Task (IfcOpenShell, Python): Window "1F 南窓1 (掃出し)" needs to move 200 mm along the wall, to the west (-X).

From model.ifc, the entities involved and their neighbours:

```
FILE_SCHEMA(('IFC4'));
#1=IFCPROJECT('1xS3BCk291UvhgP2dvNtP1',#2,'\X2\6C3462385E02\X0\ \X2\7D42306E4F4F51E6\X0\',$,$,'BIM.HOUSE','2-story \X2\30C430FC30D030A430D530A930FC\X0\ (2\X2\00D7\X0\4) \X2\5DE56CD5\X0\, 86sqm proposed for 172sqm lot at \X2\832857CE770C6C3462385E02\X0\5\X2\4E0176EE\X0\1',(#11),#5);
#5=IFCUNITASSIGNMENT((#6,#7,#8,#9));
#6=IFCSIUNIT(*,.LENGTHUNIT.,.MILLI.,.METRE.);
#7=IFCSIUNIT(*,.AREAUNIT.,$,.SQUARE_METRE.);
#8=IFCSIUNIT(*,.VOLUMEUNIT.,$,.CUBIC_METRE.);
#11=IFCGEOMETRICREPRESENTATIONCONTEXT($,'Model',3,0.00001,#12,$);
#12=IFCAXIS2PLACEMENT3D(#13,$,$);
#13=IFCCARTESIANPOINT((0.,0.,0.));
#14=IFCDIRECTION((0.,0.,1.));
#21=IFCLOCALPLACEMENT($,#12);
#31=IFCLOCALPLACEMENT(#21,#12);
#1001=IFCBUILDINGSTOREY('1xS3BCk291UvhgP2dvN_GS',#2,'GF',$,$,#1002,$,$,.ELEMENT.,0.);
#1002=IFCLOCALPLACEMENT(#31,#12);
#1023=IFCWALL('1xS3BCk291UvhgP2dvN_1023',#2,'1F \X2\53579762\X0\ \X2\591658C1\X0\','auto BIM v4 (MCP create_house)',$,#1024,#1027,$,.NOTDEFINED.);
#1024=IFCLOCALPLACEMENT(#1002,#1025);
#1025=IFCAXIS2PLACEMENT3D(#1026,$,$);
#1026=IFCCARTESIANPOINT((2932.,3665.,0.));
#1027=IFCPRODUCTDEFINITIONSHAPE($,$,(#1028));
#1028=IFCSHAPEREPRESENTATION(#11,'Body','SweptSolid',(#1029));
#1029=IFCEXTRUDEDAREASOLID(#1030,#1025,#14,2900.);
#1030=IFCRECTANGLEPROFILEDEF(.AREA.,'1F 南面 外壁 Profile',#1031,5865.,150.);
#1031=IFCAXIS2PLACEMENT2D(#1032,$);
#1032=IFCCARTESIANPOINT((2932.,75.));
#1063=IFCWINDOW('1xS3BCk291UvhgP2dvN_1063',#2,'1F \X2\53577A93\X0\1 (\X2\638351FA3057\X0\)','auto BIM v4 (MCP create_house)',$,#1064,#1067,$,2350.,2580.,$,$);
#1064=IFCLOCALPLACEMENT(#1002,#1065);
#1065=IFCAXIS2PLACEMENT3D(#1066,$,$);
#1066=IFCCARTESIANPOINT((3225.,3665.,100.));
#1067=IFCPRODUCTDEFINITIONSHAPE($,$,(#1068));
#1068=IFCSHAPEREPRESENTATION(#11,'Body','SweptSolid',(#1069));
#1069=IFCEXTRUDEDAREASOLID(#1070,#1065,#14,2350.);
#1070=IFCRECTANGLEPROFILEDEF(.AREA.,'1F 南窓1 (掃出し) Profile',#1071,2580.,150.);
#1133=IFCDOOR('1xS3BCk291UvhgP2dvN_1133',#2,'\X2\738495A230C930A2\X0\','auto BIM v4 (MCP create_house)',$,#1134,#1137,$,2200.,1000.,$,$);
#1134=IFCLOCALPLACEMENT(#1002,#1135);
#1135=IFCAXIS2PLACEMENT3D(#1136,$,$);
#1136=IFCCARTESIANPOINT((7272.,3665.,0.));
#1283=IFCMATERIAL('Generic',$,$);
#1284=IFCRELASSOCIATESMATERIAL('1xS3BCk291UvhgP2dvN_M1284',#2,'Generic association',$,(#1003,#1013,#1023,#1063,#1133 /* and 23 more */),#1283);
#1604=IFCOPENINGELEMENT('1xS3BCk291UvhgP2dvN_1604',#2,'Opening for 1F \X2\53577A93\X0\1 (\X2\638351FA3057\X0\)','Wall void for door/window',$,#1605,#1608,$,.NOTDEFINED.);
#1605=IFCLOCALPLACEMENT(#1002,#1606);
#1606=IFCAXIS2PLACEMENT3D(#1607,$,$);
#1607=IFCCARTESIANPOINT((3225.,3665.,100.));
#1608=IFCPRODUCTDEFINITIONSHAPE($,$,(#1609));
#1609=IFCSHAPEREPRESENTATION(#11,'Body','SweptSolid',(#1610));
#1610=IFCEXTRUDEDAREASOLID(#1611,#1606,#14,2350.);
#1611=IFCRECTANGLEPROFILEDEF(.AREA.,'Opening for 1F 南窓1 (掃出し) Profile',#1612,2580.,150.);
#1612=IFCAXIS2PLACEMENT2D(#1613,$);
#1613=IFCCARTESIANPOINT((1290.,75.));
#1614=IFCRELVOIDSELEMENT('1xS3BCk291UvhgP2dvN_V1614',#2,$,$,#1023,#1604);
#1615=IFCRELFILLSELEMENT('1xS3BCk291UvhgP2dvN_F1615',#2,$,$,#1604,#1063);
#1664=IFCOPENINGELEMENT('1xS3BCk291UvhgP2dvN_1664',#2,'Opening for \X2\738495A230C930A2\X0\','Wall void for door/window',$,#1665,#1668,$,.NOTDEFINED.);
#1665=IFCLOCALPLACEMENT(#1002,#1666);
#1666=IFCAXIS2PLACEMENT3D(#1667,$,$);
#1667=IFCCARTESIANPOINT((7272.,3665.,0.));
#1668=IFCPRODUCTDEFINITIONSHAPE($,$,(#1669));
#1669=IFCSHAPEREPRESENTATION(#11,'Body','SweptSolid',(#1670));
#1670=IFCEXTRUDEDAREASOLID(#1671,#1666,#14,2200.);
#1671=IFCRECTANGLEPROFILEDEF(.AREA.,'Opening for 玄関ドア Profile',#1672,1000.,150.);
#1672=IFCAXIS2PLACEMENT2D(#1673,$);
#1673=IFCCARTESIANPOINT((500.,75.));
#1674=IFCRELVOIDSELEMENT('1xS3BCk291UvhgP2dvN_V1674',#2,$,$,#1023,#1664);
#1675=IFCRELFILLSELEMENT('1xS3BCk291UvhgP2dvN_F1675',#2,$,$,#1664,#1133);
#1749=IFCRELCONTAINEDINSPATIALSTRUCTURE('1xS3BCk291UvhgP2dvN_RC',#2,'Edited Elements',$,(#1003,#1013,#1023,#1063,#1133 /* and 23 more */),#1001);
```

```python
import ifcopenshell
import ifcopenshell.api.geometry
import ifcopenshell.util.placement
import ifcopenshell.util.unit

model = ifcopenshell.open("model.ifc")
unit_scale = ifcopenshell.util.unit.calculate_unit_scale(model)

window = model.by_guid("1xS3BCk291UvhgP2dvN_1063")
opening = window.FillsVoids[0].RelatingOpeningElement
wall = opening.VoidsElements[0].RelatingBuildingElement

wall_matrix = ifcopenshell.util.placement.get_local_placement(wall.ObjectPlacement)
shift = wall_matrix[:3, 0] * -0.2 / unit_scale
before = ifcopenshell.util.placement.get_local_placement(window.ObjectPlacement)[:3, 3].copy()

# The window is not placed relative to its opening, so move both.
for product in (opening, window):
    matrix = ifcopenshell.util.placement.get_local_placement(product.ObjectPlacement)
    matrix[:3, 3] += shift
    ifcopenshell.api.geometry.edit_object_placement(model, product=product, matrix=matrix, is_si=False)

after = ifcopenshell.util.placement.get_local_placement(window.ObjectPlacement)[:3, 3]
print("window moved by", (after - before).round(3) + 0.0)

model.write("model_rev.ifc")
```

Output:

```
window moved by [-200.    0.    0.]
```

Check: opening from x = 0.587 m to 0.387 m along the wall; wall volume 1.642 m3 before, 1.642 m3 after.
